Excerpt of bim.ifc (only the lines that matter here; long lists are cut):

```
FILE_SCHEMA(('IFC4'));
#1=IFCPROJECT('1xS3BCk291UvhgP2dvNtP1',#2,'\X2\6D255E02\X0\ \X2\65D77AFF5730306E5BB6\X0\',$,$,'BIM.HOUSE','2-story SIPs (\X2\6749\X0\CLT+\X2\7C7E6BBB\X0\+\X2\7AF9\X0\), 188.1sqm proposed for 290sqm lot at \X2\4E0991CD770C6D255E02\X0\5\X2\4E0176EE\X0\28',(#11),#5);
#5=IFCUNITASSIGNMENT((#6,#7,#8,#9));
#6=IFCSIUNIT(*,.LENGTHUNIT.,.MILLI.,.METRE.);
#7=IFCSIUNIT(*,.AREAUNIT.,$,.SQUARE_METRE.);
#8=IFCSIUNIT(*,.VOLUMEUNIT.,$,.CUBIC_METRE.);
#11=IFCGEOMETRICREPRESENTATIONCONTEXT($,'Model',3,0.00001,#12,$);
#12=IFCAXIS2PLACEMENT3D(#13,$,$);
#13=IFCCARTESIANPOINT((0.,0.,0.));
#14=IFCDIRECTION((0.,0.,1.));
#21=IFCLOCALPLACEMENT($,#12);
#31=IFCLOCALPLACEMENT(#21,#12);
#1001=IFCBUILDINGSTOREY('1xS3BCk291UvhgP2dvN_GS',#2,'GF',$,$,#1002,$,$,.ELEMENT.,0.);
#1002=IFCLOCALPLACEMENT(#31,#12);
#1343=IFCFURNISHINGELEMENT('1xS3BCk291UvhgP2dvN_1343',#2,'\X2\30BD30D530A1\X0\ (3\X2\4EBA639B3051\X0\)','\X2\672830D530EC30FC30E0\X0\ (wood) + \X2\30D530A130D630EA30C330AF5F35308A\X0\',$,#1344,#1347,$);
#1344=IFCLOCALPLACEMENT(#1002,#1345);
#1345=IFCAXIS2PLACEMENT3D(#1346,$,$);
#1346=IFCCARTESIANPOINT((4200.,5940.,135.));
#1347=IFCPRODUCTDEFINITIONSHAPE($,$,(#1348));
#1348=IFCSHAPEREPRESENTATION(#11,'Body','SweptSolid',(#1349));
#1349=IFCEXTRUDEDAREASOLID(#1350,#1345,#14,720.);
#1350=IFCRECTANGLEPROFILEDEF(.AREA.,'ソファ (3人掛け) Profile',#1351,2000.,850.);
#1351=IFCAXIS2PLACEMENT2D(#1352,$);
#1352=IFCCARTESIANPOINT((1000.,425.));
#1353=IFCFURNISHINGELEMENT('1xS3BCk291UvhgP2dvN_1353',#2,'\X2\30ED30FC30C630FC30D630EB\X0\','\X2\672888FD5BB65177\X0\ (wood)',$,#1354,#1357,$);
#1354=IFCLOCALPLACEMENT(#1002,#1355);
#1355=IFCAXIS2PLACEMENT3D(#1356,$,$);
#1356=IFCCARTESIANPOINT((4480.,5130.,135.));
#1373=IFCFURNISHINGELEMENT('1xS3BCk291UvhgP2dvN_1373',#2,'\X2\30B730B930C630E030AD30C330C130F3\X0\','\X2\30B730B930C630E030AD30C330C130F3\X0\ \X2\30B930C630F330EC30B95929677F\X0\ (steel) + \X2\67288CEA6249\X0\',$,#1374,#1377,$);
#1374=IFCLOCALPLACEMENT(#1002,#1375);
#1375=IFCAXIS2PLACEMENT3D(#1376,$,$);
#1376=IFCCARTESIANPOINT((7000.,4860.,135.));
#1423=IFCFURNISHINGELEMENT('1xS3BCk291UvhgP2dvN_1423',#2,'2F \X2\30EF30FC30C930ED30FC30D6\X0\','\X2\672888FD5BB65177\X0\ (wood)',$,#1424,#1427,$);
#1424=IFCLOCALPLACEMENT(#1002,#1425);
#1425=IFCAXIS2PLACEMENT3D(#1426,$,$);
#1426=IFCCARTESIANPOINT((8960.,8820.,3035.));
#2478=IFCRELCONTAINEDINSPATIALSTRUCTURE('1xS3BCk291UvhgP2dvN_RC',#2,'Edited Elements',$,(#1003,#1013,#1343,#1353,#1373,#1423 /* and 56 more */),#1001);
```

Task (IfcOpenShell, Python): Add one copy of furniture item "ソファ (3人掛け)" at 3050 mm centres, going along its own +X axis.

```python
import ifcopenshell
import ifcopenshell.api.geometry
import ifcopenshell.api.root
import ifcopenshell.util.element
import ifcopenshell.util.placement

model = ifcopenshell.open("bim.ifc")


def reuse_history(source, copy):
    """copy_class also copies each property set's owner history, people and application; keep the originals."""
    for rel in copy.IsDefinedBy:
        if rel.is_a("IfcRelDefinesByProperties") and (history := rel.RelatingPropertyDefinition.OwnerHistory):
            rel.RelatingPropertyDefinition.OwnerHistory = source.OwnerHistory
            ifcopenshell.util.element.remove_deep2(model, history)


source = model.by_guid("1xS3BCk291UvhgP2dvN_1343")
base = ifcopenshell.util.placement.get_local_placement(source.ObjectPlacement)
step = base[:3, 0] * 3050.0

for i in range(1, 2):
    copy = ifcopenshell.api.root.copy_class(model, product=source)
    copy.Representation = ifcopenshell.util.element.copy_deep(
        model, source.Representation, exclude=["IfcGeometricRepresentationContext", "IfcRepresentationMap"]
    )
    reuse_history(source, copy)
    matrix = base.copy()
    matrix[:3, 3] += i * step
    print("added at", matrix[:3, 3].round(3) + 0.0)
    ifcopenshell.api.geometry.edit_object_placement(model, product=copy, matrix=matrix, is_si=False)

model.write("bim-out.ifc")
```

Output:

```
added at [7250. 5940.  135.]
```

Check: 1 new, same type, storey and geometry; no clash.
